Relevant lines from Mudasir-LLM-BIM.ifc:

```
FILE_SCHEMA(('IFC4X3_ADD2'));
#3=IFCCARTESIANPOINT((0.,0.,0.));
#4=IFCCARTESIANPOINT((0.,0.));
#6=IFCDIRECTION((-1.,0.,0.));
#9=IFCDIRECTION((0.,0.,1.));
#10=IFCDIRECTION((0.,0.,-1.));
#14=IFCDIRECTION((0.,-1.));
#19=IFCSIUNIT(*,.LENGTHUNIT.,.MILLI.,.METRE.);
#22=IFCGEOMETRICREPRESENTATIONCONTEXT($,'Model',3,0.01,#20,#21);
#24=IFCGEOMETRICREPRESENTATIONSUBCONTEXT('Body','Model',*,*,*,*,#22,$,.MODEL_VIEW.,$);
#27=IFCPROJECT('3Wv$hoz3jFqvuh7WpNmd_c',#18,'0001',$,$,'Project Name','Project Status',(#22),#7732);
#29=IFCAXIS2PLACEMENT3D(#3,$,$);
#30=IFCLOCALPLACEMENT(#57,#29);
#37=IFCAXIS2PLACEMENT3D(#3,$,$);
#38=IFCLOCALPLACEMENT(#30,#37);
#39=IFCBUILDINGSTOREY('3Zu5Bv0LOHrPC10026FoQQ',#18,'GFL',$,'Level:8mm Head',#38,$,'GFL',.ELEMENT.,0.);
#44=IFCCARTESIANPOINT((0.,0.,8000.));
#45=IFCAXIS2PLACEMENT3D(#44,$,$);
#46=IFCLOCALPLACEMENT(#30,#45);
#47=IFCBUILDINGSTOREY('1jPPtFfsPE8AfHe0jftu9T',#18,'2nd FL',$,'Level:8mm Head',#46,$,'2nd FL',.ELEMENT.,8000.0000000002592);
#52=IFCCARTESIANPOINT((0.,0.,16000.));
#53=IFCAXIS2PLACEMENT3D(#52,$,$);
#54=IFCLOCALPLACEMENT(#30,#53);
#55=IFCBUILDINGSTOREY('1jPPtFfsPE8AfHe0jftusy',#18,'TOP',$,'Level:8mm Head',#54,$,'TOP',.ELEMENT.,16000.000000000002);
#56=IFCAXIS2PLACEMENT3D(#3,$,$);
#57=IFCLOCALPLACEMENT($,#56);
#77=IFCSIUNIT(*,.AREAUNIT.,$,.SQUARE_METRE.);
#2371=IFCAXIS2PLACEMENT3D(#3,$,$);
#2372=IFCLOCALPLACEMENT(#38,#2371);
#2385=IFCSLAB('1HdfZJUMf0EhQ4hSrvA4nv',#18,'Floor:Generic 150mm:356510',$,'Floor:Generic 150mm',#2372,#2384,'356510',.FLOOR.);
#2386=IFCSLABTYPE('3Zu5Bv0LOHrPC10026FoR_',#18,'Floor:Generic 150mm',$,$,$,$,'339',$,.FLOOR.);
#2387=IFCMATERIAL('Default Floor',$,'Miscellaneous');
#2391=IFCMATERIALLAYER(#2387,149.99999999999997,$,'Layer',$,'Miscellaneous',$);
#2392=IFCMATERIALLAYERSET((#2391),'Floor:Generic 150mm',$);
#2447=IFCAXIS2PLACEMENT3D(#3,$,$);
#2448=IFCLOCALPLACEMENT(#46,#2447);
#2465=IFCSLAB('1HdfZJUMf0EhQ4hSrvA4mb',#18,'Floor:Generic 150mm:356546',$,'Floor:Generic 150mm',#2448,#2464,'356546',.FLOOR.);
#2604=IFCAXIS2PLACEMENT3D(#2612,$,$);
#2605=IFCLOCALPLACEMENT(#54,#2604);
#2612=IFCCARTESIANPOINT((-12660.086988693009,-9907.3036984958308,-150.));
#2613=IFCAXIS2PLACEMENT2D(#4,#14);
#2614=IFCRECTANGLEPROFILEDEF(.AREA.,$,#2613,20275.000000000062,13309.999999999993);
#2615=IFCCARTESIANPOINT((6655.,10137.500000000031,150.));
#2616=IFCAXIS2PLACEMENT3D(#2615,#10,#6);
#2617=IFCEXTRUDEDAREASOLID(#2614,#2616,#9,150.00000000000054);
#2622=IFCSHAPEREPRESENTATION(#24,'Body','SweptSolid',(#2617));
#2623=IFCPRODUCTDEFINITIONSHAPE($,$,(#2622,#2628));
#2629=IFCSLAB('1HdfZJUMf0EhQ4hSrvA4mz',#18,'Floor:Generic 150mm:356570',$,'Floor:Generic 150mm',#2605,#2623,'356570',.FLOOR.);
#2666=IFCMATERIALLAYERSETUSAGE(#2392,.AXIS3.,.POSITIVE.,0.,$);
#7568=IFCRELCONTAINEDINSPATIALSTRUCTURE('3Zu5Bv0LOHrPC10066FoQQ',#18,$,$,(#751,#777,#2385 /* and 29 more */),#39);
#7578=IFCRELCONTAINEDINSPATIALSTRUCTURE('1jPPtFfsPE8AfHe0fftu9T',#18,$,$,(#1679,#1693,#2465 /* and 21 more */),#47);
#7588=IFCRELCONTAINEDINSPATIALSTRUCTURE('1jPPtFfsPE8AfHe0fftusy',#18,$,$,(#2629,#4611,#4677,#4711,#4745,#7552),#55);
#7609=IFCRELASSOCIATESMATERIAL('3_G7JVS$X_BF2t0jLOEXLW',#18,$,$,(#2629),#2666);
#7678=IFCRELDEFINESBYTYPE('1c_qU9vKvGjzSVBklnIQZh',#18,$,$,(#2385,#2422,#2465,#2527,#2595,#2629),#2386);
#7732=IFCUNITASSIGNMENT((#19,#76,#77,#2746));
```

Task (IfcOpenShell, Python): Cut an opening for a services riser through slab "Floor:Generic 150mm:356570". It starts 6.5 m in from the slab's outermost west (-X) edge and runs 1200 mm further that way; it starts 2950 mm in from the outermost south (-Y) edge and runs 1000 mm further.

```python
import numpy as np
import ifcopenshell
import ifcopenshell.api.feature
import ifcopenshell.api.geometry
import ifcopenshell.api.root
import ifcopenshell.geom
import ifcopenshell.util.placement
import ifcopenshell.util.representation
import ifcopenshell.util.shape
import ifcopenshell.util.unit

model = ifcopenshell.open("Mudasir-LLM-BIM.ifc")
unit_scale = ifcopenshell.util.unit.calculate_unit_scale(model)
settings = ifcopenshell.geom.settings()


def volume(element):
    """Net volume in cubic metres, openings subtracted."""
    shape = ifcopenshell.geom.create_shape(settings, element)
    return ifcopenshell.util.shape.get_volume(shape.geometry)


slab = model.by_id(2629)
before = volume(slab)

# Extent in the slab's own axes, in metres. The edges named are its -X and -Y sides.
slab_shape = ifcopenshell.geom.create_shape(settings, slab)
vertices = ifcopenshell.util.shape.get_vertices(slab_shape.geometry)
x_min, y_min, bottom = vertices.min(axis=0)
top = vertices[:, 2].max()

opening = ifcopenshell.api.root.create_entity(model, ifc_class="IfcOpeningElement", name="Services riser opening", predefined_type="OPENING")
context = ifcopenshell.util.representation.get_context(model, "Model", "Body", "MODEL_VIEW")
width, depth = 1.2, 1
outline = [(0.0, 0.0), (width, 0.0), (width, depth), (0.0, depth), (0.0, 0.0)]
# Overshoot both faces by 50 mm so the cut is clean.
shape = ifcopenshell.api.geometry.add_slab_representation(
    model, context=context, depth=top - bottom + 0.1, polyline=outline
)
ifcopenshell.api.geometry.assign_representation(model, product=opening, representation=shape)

matrix = ifcopenshell.util.placement.get_local_placement(slab.ObjectPlacement)
matrix[:, 3] = matrix @ np.append(np.array([x_min + 6.5, y_min + 2.95, bottom - 0.05]) / unit_scale, 1.0)
ifcopenshell.api.geometry.edit_object_placement(model, product=opening, matrix=matrix, is_si=False)
ifcopenshell.api.feature.add_feature(model, feature=opening, element=slab)

after = volume(slab)

print(f"slab volume {before:.3f} -> {after:.3f} m3")

model.write("Mudasir-LLM-BIM_edited.ifc")
```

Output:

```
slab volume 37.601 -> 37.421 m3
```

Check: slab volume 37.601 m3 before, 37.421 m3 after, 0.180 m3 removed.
